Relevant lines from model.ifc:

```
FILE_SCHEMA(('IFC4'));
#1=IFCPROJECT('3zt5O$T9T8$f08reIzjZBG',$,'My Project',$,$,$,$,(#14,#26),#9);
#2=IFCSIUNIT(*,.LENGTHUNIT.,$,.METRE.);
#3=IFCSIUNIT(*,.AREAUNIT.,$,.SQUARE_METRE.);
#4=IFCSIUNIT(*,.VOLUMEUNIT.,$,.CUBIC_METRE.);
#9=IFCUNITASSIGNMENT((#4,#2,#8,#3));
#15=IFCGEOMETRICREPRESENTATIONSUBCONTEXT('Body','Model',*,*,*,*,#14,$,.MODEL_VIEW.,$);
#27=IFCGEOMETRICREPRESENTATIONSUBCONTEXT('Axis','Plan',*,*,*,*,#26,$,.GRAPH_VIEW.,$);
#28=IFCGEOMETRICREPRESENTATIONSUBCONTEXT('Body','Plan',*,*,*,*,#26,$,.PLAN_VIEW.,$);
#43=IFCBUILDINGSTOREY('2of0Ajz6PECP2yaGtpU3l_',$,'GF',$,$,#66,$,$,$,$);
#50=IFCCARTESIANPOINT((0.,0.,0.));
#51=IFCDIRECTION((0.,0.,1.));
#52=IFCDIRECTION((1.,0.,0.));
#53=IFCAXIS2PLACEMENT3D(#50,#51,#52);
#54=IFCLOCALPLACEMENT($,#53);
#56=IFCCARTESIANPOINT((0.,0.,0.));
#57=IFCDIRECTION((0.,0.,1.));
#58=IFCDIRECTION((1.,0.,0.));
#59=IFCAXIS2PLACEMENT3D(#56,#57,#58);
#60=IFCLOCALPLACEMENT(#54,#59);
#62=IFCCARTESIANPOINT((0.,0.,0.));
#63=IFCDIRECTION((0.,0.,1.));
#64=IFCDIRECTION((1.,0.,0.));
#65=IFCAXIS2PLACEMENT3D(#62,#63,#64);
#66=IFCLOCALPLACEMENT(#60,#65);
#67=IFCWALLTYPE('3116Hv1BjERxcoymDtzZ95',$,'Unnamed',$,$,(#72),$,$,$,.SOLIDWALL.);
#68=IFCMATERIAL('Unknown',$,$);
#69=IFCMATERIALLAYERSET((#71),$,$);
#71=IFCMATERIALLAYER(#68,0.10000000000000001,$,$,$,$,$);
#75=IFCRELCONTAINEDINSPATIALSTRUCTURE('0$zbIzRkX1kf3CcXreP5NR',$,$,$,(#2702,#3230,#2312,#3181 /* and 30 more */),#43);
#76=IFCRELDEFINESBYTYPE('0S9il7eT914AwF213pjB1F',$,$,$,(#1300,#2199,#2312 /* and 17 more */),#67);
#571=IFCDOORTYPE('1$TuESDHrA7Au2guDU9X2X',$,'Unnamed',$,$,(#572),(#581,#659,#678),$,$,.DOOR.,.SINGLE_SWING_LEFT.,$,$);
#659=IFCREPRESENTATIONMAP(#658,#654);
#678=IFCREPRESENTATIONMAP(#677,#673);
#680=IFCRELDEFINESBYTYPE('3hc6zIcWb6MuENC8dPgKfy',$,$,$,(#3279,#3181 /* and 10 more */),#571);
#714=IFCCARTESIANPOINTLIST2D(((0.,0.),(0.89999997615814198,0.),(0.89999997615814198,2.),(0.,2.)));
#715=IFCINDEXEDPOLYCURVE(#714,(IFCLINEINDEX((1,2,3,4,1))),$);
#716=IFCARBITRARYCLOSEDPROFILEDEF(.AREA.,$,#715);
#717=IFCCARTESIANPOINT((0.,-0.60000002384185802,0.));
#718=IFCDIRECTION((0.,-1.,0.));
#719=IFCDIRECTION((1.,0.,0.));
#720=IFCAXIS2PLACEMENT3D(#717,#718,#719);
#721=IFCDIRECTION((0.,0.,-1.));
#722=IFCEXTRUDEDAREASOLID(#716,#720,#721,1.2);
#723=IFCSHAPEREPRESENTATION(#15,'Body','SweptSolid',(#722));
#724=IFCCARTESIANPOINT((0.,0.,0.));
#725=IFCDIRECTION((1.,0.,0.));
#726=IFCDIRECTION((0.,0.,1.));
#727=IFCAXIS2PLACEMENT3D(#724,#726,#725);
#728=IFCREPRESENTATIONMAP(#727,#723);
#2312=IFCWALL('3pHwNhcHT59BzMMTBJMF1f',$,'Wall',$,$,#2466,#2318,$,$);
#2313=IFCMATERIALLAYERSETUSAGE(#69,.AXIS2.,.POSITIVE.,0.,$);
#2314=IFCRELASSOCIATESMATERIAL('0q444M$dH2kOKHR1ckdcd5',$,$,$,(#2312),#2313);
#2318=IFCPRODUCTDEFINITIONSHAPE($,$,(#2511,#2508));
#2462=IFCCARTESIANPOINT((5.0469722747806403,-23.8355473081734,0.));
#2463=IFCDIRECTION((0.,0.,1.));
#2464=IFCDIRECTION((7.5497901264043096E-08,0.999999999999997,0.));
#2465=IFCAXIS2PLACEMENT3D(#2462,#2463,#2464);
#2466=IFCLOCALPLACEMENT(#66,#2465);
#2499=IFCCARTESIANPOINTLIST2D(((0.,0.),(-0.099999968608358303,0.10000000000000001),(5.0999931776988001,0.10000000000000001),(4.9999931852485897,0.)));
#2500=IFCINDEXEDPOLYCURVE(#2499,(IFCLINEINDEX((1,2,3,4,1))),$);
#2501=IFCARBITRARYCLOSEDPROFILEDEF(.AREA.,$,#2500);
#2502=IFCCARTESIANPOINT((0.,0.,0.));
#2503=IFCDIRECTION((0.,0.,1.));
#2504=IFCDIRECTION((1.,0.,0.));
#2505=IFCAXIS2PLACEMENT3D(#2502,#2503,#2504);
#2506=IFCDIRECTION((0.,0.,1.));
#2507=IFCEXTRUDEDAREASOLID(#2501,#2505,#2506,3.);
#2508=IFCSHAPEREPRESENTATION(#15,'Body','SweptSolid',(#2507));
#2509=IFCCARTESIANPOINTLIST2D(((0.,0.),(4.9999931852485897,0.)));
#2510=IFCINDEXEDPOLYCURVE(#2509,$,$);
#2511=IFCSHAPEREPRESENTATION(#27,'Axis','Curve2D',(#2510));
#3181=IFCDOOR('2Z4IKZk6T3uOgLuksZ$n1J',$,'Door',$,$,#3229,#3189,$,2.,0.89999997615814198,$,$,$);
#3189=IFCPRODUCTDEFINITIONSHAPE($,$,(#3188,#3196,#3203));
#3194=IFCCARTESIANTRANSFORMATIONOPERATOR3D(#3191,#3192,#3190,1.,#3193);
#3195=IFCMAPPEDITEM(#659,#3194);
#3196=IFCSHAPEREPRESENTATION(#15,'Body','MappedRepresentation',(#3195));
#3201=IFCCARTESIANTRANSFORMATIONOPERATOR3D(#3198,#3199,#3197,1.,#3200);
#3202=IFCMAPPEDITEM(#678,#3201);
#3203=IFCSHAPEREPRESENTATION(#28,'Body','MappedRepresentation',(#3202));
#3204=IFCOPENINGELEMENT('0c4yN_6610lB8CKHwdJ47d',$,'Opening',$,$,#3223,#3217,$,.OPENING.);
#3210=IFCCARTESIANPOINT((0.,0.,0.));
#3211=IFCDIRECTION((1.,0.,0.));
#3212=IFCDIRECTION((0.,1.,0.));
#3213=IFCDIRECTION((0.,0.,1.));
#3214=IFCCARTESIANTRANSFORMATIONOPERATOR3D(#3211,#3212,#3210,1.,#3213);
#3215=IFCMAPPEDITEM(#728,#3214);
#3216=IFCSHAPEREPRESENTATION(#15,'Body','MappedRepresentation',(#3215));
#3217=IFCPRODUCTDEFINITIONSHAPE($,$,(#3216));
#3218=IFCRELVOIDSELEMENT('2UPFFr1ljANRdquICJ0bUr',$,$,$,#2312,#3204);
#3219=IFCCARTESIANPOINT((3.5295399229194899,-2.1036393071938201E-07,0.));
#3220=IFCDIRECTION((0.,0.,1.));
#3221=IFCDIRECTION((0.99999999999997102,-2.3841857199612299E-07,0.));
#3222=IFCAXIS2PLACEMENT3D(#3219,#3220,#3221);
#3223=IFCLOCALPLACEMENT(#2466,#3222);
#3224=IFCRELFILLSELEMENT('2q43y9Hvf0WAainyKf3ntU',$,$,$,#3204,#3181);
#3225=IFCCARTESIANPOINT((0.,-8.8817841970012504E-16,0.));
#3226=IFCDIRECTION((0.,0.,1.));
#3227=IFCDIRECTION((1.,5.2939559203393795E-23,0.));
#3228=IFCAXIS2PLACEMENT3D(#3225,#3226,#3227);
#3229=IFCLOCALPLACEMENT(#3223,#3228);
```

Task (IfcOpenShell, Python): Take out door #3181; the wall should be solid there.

```python
import ifcopenshell
import ifcopenshell.api.feature
import ifcopenshell.api.root
import ifcopenshell.geom
import ifcopenshell.util.shape

model = ifcopenshell.open("model.ifc")
settings = ifcopenshell.geom.settings()


def volume(element):
    """Net volume in cubic metres, openings subtracted."""
    shape = ifcopenshell.geom.create_shape(settings, element)
    return ifcopenshell.util.shape.get_volume(shape.geometry)


door = model.by_guid("2Z4IKZk6T3uOgLuksZ$n1J")
opening = door.FillsVoids[0].RelatingOpeningElement
wall = opening.VoidsElements[0].RelatingBuildingElement
before = volume(wall)

ifcopenshell.api.root.remove_product(model, product=door)
ifcopenshell.api.feature.remove_feature(model, feature=opening)

after = volume(wall)

print(f"wall volume {before:.3f} -> {after:.3f} m3")

model.write("model_v2.ifc")
```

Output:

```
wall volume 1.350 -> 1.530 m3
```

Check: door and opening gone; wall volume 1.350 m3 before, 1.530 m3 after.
